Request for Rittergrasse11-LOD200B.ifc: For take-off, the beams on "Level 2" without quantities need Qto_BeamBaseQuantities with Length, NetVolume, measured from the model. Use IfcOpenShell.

First a look at what the model holds.

```python
import ifcopenshell
import ifcopenshell.util.element
import ifcopenshell.util.unit

model = ifcopenshell.open("Rittergrasse11-LOD200B.ifc")
print(model.schema)
for unit_type in ("LENGTHUNIT", "AREAUNIT", "VOLUMEUNIT"):
    print(unit_type, ifcopenshell.util.unit.calculate_unit_scale(model, unit_type))
storey = next(s for s in model.by_type("IfcBuildingStorey") if s.Name == "Level 2")
beams = [e for e in ifcopenshell.util.element.get_decomposition(storey) if e.is_a("IfcBeam")]
for e in sorted(beams, key=lambda e: e.id()):
    print(e.id(), e.is_a(), e.Name, list(ifcopenshell.util.element.get_psets(e, qtos_only=True)), sep=" | ")
```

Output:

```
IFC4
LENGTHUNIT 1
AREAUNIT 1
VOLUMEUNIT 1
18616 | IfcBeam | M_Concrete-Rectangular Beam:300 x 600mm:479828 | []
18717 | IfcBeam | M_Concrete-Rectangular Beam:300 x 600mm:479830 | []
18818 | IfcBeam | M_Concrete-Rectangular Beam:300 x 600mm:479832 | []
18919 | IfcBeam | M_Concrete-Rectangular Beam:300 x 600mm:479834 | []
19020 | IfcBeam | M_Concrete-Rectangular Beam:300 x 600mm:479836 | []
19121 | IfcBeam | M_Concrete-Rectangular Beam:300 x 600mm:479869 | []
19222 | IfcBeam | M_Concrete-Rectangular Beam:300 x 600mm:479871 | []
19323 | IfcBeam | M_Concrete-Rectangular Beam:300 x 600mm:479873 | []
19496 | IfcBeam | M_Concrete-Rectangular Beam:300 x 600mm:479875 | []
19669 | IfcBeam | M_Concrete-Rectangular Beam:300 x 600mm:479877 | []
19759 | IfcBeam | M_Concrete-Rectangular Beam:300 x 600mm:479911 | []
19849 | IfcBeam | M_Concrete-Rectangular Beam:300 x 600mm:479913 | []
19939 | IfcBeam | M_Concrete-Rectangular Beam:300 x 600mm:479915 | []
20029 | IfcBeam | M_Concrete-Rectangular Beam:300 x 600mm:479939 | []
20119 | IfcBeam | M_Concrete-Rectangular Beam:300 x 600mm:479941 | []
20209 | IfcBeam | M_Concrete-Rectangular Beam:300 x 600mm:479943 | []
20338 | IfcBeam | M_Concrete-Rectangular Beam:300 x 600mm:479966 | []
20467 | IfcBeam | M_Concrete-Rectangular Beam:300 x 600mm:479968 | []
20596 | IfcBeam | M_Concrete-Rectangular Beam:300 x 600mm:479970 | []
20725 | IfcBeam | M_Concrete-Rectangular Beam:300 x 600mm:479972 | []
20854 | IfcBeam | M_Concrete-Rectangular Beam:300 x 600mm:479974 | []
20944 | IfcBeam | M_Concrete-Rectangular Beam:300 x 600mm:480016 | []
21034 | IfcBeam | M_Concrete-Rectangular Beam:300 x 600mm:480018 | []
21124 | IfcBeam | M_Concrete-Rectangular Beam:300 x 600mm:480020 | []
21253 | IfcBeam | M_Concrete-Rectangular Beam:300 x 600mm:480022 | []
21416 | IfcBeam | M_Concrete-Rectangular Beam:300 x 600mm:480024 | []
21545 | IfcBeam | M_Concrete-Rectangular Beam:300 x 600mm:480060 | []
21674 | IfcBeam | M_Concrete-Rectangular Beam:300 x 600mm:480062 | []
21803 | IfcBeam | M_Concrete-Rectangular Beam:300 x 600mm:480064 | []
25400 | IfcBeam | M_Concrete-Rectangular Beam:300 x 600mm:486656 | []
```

```python
import ifcopenshell
import ifcopenshell.api.pset
import ifcopenshell.geom
import ifcopenshell.util.element
import ifcopenshell.util.shape
import ifcopenshell.util.unit

model = ifcopenshell.open("Rittergrasse11-LOD200B.ifc")
unit_scale = ifcopenshell.util.unit.calculate_unit_scale(model)
volume_scale = ifcopenshell.util.unit.calculate_unit_scale(model, "VOLUMEUNIT")
settings = ifcopenshell.geom.settings()

storey = next(s for s in model.by_type("IfcBuildingStorey") if s.Name == "Level 2")
beams = [e for e in ifcopenshell.util.element.get_decomposition(storey) if e.is_a("IfcBeam")]

for e in sorted(beams, key=lambda e: e.id()):
    if ifcopenshell.util.element.get_psets(e, qtos_only=True, should_inherit=False):
        continue
    # Geometry comes back in metres, in the element's own axes.
    shape = ifcopenshell.geom.create_shape(settings, e)
    values = {
        "Length": ifcopenshell.util.shape.get_max_xyz(shape.geometry) / unit_scale,
        "NetVolume": ifcopenshell.util.shape.get_volume(shape.geometry) / volume_scale,
    }
    qto = ifcopenshell.api.pset.add_qto(model, product=e, name="Qto_BeamBaseQuantities")
    ifcopenshell.api.pset.edit_qto(model, qto=qto, properties=values)
    print(e.id(), {k: round(v, 3) for k, v in values.items()})

model.write("Rittergrasse11-LOD200B_edited.ifc")
```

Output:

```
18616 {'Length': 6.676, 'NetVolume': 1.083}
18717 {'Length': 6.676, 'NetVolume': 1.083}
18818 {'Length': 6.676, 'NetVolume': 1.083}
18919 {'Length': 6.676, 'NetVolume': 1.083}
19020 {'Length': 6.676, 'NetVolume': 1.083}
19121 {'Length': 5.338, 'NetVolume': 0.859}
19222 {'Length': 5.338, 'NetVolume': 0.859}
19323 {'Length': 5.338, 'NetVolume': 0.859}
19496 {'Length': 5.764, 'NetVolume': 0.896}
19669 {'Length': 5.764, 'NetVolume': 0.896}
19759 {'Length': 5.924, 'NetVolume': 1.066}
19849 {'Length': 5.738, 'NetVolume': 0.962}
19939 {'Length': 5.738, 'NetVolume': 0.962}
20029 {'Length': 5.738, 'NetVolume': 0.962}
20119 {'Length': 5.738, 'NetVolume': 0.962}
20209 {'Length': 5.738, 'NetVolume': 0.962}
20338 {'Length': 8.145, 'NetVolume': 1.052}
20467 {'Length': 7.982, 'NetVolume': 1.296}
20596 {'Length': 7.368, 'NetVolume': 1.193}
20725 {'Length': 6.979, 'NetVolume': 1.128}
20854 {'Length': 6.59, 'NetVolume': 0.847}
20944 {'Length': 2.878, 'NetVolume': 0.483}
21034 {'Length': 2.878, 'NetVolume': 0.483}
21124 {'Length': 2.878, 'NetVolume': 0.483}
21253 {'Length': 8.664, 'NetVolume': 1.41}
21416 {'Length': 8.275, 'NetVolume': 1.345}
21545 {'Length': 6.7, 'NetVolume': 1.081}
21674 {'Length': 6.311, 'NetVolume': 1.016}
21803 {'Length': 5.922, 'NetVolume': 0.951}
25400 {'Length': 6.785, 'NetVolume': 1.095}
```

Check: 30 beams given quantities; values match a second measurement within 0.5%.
